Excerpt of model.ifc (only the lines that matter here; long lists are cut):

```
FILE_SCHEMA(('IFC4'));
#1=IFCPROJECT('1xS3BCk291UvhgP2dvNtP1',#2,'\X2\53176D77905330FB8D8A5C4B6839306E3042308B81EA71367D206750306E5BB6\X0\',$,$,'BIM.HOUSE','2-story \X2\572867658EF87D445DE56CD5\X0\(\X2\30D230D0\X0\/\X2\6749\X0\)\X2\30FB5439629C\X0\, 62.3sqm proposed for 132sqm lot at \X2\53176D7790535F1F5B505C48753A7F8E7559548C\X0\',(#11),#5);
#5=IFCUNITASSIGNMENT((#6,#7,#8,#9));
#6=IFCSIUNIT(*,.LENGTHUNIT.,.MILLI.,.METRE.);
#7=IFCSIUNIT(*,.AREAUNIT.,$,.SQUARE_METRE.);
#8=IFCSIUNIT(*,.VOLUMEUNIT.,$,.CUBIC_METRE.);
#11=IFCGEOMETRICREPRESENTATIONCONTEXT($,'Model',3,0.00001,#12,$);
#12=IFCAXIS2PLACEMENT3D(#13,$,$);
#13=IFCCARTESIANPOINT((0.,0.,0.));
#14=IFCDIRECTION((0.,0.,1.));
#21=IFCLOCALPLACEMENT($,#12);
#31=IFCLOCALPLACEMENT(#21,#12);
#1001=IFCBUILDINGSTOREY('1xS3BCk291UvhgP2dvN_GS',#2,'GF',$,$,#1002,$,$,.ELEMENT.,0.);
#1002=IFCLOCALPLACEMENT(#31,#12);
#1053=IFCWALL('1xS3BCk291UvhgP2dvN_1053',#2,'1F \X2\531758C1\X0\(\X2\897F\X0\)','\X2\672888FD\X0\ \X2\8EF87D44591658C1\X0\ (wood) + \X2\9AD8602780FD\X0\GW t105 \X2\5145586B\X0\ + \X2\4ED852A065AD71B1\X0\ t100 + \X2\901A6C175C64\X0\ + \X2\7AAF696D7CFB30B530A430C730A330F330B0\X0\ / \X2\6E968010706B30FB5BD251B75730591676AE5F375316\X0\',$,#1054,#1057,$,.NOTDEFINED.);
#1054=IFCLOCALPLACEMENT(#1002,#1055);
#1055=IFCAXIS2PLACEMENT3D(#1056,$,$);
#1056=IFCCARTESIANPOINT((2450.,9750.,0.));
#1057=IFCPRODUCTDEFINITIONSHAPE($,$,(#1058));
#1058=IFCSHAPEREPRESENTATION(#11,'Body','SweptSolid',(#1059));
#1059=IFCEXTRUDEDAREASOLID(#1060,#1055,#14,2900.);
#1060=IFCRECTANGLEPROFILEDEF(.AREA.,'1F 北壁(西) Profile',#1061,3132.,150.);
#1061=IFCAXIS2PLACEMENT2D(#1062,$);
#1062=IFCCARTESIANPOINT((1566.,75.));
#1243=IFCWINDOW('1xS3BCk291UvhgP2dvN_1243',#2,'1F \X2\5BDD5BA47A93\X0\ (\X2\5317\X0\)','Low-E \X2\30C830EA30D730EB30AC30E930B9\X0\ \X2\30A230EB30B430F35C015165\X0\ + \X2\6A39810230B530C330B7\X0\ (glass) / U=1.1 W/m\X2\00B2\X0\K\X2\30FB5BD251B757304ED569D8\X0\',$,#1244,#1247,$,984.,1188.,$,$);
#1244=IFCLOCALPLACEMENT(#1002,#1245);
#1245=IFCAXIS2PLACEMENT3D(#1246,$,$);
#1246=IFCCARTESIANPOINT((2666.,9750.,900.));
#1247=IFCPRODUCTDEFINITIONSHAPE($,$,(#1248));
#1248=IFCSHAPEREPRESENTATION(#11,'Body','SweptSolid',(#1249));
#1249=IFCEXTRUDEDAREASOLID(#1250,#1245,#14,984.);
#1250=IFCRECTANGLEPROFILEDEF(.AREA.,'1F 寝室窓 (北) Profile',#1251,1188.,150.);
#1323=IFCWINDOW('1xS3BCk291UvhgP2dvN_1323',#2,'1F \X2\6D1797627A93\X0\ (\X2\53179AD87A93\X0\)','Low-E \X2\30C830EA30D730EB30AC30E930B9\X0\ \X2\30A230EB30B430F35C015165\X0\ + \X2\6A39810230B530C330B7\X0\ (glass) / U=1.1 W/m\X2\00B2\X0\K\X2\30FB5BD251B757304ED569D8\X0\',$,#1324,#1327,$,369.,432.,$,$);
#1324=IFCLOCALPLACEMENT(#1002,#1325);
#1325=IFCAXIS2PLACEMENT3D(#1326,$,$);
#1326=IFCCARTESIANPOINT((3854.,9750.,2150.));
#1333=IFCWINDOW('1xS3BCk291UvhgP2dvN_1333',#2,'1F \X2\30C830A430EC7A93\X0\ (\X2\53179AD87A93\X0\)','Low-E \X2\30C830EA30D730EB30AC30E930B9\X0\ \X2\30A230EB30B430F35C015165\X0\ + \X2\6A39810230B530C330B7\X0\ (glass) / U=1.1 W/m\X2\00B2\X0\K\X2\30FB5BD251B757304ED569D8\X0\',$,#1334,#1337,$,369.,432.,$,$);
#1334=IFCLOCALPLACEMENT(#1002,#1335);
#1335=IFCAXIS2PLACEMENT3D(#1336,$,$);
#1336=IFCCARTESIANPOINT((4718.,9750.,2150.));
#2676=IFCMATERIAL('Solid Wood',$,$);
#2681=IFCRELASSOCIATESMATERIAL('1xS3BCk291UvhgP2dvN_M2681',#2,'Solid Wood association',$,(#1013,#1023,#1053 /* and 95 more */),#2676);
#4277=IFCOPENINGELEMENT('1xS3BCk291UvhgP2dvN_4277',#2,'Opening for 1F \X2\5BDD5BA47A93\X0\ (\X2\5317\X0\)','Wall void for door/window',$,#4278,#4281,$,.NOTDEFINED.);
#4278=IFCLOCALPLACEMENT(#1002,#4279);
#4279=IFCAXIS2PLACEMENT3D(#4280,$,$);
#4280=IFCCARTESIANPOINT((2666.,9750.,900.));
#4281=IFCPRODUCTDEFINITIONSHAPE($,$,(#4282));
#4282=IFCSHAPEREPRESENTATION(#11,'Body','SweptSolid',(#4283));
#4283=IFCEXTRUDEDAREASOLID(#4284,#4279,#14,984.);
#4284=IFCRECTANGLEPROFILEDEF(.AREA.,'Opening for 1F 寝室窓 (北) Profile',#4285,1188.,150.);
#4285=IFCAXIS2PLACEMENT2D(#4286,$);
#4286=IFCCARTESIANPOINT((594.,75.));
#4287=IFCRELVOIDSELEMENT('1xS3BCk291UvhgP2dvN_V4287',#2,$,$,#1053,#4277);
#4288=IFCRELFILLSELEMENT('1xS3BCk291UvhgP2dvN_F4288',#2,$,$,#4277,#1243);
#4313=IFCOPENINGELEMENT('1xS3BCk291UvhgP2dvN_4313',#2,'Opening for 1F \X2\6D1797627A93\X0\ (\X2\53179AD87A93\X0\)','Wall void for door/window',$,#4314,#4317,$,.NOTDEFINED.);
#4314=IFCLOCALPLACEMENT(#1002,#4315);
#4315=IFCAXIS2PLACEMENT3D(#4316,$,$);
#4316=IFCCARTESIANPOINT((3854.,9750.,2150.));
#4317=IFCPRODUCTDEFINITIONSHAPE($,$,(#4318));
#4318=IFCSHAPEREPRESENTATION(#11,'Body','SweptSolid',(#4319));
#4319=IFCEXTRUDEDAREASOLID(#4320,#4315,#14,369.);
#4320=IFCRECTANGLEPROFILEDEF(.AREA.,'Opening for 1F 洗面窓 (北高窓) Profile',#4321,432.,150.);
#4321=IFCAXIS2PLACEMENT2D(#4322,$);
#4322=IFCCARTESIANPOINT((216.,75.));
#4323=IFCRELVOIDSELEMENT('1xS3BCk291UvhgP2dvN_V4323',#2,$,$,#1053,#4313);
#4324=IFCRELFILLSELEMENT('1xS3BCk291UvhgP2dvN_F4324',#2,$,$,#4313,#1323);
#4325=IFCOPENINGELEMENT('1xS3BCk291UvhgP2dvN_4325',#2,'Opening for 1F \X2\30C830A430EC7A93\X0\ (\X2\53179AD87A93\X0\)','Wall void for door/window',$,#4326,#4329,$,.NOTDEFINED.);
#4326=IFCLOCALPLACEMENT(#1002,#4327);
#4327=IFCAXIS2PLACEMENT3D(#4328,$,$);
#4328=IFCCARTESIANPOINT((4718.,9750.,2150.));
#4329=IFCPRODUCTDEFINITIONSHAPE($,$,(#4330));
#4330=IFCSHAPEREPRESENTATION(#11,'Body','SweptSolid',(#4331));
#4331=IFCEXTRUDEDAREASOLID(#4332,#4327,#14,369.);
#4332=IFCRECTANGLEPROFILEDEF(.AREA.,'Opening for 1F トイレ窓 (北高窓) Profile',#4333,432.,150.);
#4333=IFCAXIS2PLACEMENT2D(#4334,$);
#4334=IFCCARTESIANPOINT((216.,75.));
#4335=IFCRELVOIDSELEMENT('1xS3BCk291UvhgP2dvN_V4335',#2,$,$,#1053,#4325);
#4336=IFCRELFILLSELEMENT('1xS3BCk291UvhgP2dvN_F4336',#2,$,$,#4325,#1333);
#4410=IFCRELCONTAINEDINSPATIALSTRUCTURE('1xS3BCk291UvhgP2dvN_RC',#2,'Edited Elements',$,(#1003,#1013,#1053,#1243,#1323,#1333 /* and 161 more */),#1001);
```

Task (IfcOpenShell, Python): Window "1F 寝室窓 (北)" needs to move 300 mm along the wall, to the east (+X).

```python
import ifcopenshell
import ifcopenshell.api.geometry
import ifcopenshell.util.placement

model = ifcopenshell.open("model.ifc")

window = model.by_guid("1xS3BCk291UvhgP2dvN_1243")
opening = window.FillsVoids[0].RelatingOpeningElement
wall = opening.VoidsElements[0].RelatingBuildingElement

wall_matrix = ifcopenshell.util.placement.get_local_placement(wall.ObjectPlacement)
shift = wall_matrix[:3, 0] * 300.0
before = ifcopenshell.util.placement.get_local_placement(window.ObjectPlacement)[:3, 3].copy()

# The window is not placed relative to its opening, so move both.
for product in (opening, window):
    matrix = ifcopenshell.util.placement.get_local_placement(product.ObjectPlacement)
    matrix[:3, 3] += shift
    ifcopenshell.api.geometry.edit_object_placement(model, product=product, matrix=matrix, is_si=False)

after = ifcopenshell.util.placement.get_local_placement(window.ObjectPlacement)[:3, 3]
print("window moved by", (after - before).round(3) + 0.0)

model.write("model_updated.ifc")
```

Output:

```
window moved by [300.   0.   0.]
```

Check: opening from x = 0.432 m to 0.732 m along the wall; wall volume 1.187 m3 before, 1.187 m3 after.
